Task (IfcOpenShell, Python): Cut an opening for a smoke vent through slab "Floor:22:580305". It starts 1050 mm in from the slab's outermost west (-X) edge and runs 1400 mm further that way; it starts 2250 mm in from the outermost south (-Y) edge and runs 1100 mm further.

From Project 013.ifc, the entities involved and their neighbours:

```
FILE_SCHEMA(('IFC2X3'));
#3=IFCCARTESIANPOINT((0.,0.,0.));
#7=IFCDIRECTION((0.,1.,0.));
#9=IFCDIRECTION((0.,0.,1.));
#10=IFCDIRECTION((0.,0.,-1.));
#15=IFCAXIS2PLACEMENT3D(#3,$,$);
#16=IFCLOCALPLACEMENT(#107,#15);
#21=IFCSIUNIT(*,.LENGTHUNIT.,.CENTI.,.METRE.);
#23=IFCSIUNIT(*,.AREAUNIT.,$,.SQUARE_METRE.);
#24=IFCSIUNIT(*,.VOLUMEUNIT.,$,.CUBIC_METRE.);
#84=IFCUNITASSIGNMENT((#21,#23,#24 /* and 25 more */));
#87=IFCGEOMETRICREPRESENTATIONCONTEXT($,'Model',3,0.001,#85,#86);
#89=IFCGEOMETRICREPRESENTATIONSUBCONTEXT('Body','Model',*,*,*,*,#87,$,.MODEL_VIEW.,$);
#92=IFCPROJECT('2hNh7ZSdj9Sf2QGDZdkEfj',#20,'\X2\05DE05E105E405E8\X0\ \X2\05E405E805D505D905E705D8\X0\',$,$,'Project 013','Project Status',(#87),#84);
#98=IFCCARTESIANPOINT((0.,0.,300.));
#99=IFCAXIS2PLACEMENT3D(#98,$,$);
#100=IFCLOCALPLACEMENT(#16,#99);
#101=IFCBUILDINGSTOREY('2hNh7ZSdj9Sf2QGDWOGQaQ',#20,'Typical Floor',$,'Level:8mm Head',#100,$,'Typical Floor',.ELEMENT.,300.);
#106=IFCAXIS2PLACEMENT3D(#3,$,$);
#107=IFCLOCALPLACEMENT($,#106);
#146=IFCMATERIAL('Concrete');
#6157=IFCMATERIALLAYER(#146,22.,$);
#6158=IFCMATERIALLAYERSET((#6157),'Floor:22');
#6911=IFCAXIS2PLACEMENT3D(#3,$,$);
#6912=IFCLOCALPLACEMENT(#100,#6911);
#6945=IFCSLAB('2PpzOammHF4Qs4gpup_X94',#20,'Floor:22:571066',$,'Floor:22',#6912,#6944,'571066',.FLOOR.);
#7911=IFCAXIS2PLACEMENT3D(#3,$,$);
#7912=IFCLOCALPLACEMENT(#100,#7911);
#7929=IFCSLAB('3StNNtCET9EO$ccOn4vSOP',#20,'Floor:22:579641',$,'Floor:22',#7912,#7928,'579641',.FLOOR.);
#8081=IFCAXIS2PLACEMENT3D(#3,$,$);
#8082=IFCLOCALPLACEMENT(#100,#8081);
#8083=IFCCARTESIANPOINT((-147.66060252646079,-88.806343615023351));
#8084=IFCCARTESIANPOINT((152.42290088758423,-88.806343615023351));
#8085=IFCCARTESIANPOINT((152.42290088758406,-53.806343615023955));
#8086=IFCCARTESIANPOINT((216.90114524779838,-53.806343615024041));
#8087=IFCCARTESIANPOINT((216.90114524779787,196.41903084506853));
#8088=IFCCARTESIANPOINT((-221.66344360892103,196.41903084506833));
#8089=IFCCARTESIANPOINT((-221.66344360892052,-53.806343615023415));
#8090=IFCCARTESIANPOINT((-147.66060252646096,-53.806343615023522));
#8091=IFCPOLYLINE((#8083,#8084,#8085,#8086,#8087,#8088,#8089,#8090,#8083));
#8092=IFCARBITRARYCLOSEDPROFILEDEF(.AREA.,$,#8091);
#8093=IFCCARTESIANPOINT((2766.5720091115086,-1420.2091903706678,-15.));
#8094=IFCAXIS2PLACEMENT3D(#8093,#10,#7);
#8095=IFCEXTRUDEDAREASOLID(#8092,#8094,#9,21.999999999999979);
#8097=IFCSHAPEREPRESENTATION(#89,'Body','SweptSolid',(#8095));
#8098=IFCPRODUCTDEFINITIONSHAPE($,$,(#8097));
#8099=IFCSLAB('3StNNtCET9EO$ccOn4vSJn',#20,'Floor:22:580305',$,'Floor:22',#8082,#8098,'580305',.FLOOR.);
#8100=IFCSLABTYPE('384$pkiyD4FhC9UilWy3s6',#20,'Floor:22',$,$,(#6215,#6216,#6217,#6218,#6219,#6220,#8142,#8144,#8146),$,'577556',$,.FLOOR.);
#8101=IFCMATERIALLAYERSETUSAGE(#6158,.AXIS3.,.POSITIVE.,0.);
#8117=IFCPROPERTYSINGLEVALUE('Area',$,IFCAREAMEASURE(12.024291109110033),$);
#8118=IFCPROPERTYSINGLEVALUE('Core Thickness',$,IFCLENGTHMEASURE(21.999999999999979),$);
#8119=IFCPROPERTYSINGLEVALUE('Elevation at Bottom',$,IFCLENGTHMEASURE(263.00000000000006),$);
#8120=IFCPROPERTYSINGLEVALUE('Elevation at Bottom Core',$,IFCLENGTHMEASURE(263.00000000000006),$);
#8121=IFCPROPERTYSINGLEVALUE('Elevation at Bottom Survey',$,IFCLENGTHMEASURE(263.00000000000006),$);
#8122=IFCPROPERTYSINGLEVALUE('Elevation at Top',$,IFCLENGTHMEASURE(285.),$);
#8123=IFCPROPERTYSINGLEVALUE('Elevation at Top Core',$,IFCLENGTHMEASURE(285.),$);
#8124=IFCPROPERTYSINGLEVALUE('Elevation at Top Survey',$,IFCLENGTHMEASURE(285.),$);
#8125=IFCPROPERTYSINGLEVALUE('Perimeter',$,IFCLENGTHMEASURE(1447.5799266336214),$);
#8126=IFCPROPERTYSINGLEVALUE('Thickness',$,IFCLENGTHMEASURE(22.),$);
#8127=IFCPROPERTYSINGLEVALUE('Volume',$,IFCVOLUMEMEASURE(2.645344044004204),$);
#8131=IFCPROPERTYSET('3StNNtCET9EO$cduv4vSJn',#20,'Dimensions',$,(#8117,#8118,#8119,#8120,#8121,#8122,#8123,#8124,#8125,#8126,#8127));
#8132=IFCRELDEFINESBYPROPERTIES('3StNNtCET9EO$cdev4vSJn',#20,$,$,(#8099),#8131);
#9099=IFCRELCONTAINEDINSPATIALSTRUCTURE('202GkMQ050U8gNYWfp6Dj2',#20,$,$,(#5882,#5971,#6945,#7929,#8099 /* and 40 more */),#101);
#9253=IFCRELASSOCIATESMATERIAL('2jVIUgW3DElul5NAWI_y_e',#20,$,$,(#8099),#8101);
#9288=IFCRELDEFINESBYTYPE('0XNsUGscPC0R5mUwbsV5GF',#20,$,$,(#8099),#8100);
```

```python
import numpy as np
import ifcopenshell
import ifcopenshell.api.feature
import ifcopenshell.api.geometry
import ifcopenshell.api.pset
import ifcopenshell.api.root
import ifcopenshell.geom
import ifcopenshell.util.element
import ifcopenshell.util.placement
import ifcopenshell.util.representation
import ifcopenshell.util.shape
import ifcopenshell.util.unit

model = ifcopenshell.open("Project 013.ifc")
unit_scale = ifcopenshell.util.unit.calculate_unit_scale(model)
area_scale = ifcopenshell.util.unit.calculate_unit_scale(model, "AREAUNIT")
volume_scale = ifcopenshell.util.unit.calculate_unit_scale(model, "VOLUMEUNIT")
settings = ifcopenshell.geom.settings()


def volume(element):
    """Net volume in cubic metres, openings subtracted."""
    shape = ifcopenshell.geom.create_shape(settings, element)
    return ifcopenshell.util.shape.get_volume(shape.geometry)


slab = model.by_guid("3StNNtCET9EO$ccOn4vSJn")
before = volume(slab)

# Extent in the slab's own axes, in metres. The edges named are its -X and -Y sides.
slab_shape = ifcopenshell.geom.create_shape(settings, slab)
vertices = ifcopenshell.util.shape.get_vertices(slab_shape.geometry)
x_min, y_min, bottom = vertices.min(axis=0)
top = vertices[:, 2].max()

opening = ifcopenshell.api.root.create_entity(model, ifc_class="IfcOpeningElement", name="Smoke vent opening")
context = ifcopenshell.util.representation.get_context(model, "Model", "Body", "MODEL_VIEW")
width, depth = 1.4, 1.1
outline = [(0.0, 0.0), (width, 0.0), (width, depth), (0.0, depth), (0.0, 0.0)]
# Overshoot both faces by 50 mm so the cut is clean.
shape = ifcopenshell.api.geometry.add_slab_representation(
    model, context=context, depth=top - bottom + 0.1, polyline=outline
)
ifcopenshell.api.geometry.assign_representation(model, product=opening, representation=shape)

matrix = ifcopenshell.util.placement.get_local_placement(slab.ObjectPlacement)
matrix[:, 3] = matrix @ np.append(np.array([x_min + 1.05, y_min + 2.25, bottom - 0.05]) / unit_scale, 1.0)
ifcopenshell.api.geometry.edit_object_placement(model, product=opening, matrix=matrix, is_si=False)
ifcopenshell.api.feature.add_feature(model, feature=opening, element=slab)

after = volume(slab)

# Update the slab's stored quantities.
pset = model.by_id(ifcopenshell.util.element.get_pset(slab, "Dimensions", should_inherit=False)["id"])
ifcopenshell.api.pset.edit_pset(model, pset=pset, properties={
    "Area": model.create_entity("IfcAreaMeasure", after / (top - bottom) / area_scale),
    "Volume": model.create_entity("IfcVolumeMeasure", after / volume_scale),
})

print(f"slab volume {before:.3f} -> {after:.3f} m3")

model.write("Project 013-out.ifc")
```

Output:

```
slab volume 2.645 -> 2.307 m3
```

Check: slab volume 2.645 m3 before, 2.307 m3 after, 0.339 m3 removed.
